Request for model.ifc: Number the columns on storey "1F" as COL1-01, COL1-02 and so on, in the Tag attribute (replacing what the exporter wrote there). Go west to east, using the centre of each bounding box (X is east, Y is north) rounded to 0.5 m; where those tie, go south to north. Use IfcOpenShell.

First a look at what the model holds.

```python
import ifcopenshell
import ifcopenshell.util.element
import ifcopenshell.util.placement

model = ifcopenshell.open("model.ifc")
print(model.schema)
storey = next(s for s in model.by_type("IfcBuildingStorey") if s.Name == "1F")
columns = [e for e in ifcopenshell.util.element.get_decomposition(storey) if e.is_a("IfcColumn")]
for e in sorted(columns, key=lambda e: e.id()):
    origin = ifcopenshell.util.placement.get_local_placement(e.ObjectPlacement)[:3, 3]
    print(e.id(), e.Tag, e.Name, origin.round(2) + 0.0, sep=" | ")
```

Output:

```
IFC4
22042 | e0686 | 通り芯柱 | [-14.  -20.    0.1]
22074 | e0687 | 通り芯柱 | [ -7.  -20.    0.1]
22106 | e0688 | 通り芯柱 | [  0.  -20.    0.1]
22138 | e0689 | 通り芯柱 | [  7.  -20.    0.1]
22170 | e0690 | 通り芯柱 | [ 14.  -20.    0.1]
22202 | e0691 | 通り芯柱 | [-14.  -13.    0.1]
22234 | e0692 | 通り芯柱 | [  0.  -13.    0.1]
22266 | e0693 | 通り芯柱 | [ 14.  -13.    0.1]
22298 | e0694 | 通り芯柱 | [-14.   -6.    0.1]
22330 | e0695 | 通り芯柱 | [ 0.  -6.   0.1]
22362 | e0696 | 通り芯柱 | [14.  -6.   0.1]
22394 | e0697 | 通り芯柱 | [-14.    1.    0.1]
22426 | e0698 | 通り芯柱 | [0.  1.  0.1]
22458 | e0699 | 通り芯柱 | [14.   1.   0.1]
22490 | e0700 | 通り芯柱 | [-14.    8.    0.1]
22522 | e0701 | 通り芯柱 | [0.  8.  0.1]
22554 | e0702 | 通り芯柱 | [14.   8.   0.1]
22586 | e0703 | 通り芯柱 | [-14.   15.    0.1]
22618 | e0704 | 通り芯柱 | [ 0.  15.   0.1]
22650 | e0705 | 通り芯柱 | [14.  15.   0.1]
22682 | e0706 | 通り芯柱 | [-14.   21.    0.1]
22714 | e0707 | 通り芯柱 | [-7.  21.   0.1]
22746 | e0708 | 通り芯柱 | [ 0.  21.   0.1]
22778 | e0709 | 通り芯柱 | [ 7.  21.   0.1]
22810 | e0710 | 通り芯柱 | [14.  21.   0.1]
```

```python
import ifcopenshell
import ifcopenshell.geom
import ifcopenshell.util.element
import ifcopenshell.util.shape

model = ifcopenshell.open("model.ifc")
settings = ifcopenshell.geom.settings()
settings.set("use-world-coords", True)


def centre(element):
    shape = ifcopenshell.geom.create_shape(settings, element)
    return ifcopenshell.util.shape.get_bbox_centroid(shape.geometry)


storey = next(s for s in model.by_type("IfcBuildingStorey") if s.Name == "1F")
columns = [e for e in ifcopenshell.util.element.get_decomposition(storey) if e.is_a("IfcColumn")]

# Insertion points can sit at a corner or the storey origin, so sort by the geometry (in metres).
centres = {e: centre(e) for e in columns}
columns.sort(key=lambda e: (round(centres[e][0] / 0.5), centres[e][1]))

for i, e in enumerate(columns, start=1):
    number = f"COL1-{i:02d}"
    e.Tag = number
    print(e.id(), number)

model.write("model-out.ifc")
```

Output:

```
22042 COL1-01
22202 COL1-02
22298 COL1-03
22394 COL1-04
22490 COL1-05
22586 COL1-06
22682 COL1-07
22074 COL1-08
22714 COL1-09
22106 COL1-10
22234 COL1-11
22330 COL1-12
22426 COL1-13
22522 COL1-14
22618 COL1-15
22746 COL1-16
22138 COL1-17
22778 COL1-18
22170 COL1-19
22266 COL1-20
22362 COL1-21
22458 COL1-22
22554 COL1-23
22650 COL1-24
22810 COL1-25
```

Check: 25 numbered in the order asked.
